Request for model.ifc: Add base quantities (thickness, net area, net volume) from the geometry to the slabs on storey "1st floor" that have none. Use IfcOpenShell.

First a look at what the model holds.

```python
import ifcopenshell
import ifcopenshell.util.element
import ifcopenshell.util.unit

model = ifcopenshell.open("model.ifc")
print(model.schema)
for unit_type in ("LENGTHUNIT", "AREAUNIT", "VOLUMEUNIT"):
    print(unit_type, ifcopenshell.util.unit.calculate_unit_scale(model, unit_type))
storey = next(s for s in model.by_type("IfcBuildingStorey") if s.Name == "1st floor")
slabs = [e for e in ifcopenshell.util.element.get_decomposition(storey) if e.is_a("IfcSlab")]
for e in sorted(slabs, key=lambda e: e.id()):
    print(e.id(), e.is_a(), e.Name, list(ifcopenshell.util.element.get_psets(e, qtos_only=True)), sep=" | ")
```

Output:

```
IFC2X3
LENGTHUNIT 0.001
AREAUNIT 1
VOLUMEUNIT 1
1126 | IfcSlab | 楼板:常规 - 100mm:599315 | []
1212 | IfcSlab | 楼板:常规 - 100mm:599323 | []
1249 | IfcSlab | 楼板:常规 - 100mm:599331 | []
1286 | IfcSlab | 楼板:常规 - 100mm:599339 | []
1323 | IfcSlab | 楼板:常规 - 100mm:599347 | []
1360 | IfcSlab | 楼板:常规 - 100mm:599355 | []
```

```python
import ifcopenshell
import ifcopenshell.api.pset
import ifcopenshell.geom
import ifcopenshell.util.element
import ifcopenshell.util.shape
import ifcopenshell.util.unit

model = ifcopenshell.open("model.ifc")
unit_scale = ifcopenshell.util.unit.calculate_unit_scale(model)
area_scale = ifcopenshell.util.unit.calculate_unit_scale(model, "AREAUNIT")
volume_scale = ifcopenshell.util.unit.calculate_unit_scale(model, "VOLUMEUNIT")
settings = ifcopenshell.geom.settings()

storey = next(s for s in model.by_type("IfcBuildingStorey") if s.Name == "1st floor")
slabs = [e for e in ifcopenshell.util.element.get_decomposition(storey) if e.is_a("IfcSlab")]

for e in sorted(slabs, key=lambda e: e.id()):
    if ifcopenshell.util.element.get_psets(e, qtos_only=True, should_inherit=False):
        continue
    # Geometry comes back in metres, in the element's own axes.
    shape = ifcopenshell.geom.create_shape(settings, e)
    values = {
        "Width": ifcopenshell.util.shape.get_z(shape.geometry) / unit_scale,
        "NetArea": ifcopenshell.util.shape.get_footprint_area(shape.geometry) / area_scale,
        "NetVolume": ifcopenshell.util.shape.get_volume(shape.geometry) / volume_scale,
    }
    qto = ifcopenshell.api.pset.add_qto(model, product=e, name="BaseQuantities")
    ifcopenshell.api.pset.edit_qto(model, qto=qto, properties=values)
    print(e.id(), {k: round(v, 3) for k, v in values.items()})

model.write("model_rev.ifc")
```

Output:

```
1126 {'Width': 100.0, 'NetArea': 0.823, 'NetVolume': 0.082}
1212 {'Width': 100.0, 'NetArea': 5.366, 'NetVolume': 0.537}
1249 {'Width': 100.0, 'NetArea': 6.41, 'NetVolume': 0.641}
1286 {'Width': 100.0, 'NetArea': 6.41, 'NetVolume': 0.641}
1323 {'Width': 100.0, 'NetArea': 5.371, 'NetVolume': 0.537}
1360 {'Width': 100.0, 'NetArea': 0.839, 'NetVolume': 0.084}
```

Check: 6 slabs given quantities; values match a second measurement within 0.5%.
